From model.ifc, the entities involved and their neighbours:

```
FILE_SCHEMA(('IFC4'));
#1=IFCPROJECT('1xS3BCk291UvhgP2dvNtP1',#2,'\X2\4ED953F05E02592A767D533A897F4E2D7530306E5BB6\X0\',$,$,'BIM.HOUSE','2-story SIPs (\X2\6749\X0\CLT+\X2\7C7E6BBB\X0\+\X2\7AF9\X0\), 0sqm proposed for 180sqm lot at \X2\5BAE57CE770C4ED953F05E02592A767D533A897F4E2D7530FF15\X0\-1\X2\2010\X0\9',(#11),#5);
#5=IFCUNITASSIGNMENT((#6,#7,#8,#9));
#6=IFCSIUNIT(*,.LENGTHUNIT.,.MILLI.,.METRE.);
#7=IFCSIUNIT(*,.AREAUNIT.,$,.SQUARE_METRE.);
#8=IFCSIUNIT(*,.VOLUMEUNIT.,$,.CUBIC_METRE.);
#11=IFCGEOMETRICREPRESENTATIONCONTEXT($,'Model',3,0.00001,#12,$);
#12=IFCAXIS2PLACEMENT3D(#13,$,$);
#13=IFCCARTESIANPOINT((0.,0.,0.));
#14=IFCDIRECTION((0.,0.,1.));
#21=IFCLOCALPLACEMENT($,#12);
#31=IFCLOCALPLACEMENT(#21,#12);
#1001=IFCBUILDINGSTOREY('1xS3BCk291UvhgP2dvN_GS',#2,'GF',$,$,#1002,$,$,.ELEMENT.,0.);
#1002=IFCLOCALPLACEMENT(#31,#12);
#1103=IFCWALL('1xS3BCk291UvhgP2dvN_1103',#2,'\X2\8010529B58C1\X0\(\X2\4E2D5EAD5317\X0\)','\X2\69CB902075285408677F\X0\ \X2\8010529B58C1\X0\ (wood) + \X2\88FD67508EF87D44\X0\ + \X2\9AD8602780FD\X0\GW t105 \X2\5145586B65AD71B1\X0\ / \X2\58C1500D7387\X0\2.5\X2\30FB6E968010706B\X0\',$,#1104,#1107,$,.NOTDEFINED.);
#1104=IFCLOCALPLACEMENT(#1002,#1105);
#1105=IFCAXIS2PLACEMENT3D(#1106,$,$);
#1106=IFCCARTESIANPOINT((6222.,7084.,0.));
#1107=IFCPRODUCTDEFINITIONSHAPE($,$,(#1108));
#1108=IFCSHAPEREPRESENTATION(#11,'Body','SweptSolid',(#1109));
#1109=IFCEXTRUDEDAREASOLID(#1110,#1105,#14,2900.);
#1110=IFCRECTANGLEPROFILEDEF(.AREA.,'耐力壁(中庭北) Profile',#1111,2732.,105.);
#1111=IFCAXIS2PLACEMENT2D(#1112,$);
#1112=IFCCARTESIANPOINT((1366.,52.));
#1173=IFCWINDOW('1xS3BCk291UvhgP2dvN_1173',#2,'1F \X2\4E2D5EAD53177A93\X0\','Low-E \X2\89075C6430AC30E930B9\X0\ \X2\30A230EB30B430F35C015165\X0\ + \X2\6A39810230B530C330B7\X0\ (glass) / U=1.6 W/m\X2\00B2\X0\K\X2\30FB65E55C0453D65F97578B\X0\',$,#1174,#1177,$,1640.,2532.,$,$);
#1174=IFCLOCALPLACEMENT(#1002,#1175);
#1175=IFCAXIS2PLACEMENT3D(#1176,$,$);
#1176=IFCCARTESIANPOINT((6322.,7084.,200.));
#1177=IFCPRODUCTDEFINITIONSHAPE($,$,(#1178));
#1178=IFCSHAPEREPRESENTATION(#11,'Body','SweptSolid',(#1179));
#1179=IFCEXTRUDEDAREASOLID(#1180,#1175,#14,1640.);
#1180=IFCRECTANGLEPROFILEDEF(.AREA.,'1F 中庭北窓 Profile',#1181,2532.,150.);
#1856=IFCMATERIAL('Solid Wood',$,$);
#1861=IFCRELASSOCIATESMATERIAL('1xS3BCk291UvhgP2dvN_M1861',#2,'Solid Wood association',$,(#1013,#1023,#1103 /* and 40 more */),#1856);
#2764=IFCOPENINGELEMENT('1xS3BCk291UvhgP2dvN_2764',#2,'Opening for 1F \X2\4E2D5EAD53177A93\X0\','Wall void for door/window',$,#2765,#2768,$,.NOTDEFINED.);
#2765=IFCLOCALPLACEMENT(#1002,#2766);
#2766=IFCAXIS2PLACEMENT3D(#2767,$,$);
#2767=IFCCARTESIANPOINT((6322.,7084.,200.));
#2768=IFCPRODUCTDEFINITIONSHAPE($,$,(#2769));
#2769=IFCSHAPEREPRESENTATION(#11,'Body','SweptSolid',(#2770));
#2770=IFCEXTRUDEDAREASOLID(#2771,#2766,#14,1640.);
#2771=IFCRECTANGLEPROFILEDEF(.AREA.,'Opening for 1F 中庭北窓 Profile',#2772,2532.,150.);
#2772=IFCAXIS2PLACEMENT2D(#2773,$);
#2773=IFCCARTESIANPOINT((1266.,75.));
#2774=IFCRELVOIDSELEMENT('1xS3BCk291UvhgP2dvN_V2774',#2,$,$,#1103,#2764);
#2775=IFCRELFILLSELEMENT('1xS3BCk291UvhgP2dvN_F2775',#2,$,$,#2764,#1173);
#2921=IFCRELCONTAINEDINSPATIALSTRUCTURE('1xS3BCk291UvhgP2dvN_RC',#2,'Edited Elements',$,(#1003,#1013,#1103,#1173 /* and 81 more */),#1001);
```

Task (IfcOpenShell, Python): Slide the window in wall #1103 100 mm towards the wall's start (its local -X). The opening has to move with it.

```python
import ifcopenshell
import ifcopenshell.api.geometry
import ifcopenshell.util.placement
import ifcopenshell.util.unit

model = ifcopenshell.open("model.ifc")
unit_scale = ifcopenshell.util.unit.calculate_unit_scale(model)

window = model.by_guid("1xS3BCk291UvhgP2dvN_1173")
opening = window.FillsVoids[0].RelatingOpeningElement
wall = opening.VoidsElements[0].RelatingBuildingElement

wall_matrix = ifcopenshell.util.placement.get_local_placement(wall.ObjectPlacement)
shift = wall_matrix[:3, 0] * -0.1 / unit_scale
before = ifcopenshell.util.placement.get_local_placement(window.ObjectPlacement)[:3, 3].copy()

# The window is not placed relative to its opening, so move both.
for product in (opening, window):
    matrix = ifcopenshell.util.placement.get_local_placement(product.ObjectPlacement)
    matrix[:3, 3] += shift
    ifcopenshell.api.geometry.edit_object_placement(model, product=product, matrix=matrix, is_si=False)

after = ifcopenshell.util.placement.get_local_placement(window.ObjectPlacement)[:3, 3]
print("window moved by", (after - before).round(3) + 0.0)

model.write("model_updated.ifc")
```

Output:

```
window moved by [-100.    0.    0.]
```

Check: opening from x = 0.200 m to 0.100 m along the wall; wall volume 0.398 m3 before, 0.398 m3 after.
